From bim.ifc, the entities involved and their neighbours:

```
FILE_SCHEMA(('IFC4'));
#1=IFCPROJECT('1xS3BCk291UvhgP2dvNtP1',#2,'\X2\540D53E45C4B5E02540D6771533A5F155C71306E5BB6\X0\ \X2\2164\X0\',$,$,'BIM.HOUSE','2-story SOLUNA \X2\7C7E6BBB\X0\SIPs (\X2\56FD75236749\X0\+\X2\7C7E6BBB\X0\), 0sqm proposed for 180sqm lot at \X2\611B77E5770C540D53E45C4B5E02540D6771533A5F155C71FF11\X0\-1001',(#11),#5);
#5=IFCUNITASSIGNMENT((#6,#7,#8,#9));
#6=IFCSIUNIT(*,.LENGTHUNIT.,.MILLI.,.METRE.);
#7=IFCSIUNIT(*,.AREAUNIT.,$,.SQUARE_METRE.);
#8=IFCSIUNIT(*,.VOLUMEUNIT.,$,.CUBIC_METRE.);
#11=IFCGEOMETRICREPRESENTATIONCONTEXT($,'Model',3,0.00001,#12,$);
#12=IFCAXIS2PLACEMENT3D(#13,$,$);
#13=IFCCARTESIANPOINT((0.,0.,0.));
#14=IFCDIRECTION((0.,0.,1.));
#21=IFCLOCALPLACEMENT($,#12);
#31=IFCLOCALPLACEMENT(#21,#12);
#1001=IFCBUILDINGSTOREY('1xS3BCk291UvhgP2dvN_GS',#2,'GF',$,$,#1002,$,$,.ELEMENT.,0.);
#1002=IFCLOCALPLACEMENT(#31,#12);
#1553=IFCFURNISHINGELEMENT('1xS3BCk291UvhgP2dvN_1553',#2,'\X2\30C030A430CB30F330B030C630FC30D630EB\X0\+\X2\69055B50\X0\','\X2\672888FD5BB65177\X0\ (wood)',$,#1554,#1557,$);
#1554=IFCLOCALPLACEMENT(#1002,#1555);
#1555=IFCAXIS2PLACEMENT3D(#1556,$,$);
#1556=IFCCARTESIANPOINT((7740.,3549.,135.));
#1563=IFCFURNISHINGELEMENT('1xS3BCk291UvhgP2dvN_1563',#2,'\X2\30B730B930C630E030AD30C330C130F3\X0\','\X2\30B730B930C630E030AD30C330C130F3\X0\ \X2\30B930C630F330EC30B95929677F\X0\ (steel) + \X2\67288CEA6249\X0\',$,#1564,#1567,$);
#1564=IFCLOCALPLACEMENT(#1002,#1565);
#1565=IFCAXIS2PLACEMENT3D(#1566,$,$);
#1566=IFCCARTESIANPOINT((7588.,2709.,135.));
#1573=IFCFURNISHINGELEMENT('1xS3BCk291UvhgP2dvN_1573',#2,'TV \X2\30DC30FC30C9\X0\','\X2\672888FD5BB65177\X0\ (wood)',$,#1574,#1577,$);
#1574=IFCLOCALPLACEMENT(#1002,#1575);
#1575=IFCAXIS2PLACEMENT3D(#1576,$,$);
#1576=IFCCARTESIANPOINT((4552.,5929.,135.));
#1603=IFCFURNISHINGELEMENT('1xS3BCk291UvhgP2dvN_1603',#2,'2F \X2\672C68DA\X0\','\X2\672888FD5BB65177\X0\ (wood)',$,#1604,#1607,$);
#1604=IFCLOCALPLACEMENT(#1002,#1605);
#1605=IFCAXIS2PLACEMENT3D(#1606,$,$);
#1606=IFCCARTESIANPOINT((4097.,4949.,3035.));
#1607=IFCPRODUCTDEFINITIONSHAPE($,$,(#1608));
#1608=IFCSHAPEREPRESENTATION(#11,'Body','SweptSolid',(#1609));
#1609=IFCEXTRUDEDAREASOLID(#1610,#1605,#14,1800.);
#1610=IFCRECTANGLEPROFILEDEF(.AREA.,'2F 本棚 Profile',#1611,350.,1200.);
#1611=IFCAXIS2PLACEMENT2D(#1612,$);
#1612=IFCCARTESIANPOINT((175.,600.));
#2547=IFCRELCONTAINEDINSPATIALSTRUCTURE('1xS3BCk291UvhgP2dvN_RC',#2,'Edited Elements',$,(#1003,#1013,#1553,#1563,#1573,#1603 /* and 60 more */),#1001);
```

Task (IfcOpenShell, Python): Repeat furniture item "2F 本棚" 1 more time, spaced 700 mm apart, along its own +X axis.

```python
import ifcopenshell
import ifcopenshell.api.geometry
import ifcopenshell.api.root
import ifcopenshell.util.element
import ifcopenshell.util.placement
import ifcopenshell.util.unit

model = ifcopenshell.open("bim.ifc")
unit_scale = ifcopenshell.util.unit.calculate_unit_scale(model)


def reuse_history(source, copy):
    """copy_class also copies each property set's owner history, people and application; keep the originals."""
    for rel in copy.IsDefinedBy:
        if rel.is_a("IfcRelDefinesByProperties") and (history := rel.RelatingPropertyDefinition.OwnerHistory):
            rel.RelatingPropertyDefinition.OwnerHistory = source.OwnerHistory
            ifcopenshell.util.element.remove_deep2(model, history)


source = model.by_guid("1xS3BCk291UvhgP2dvN_1603")
base = ifcopenshell.util.placement.get_local_placement(source.ObjectPlacement)
step = base[:3, 0] * 0.7 / unit_scale

for i in range(1, 2):
    copy = ifcopenshell.api.root.copy_class(model, product=source)
    copy.Representation = ifcopenshell.util.element.copy_deep(
        model, source.Representation, exclude=["IfcGeometricRepresentationContext", "IfcRepresentationMap"]
    )
    reuse_history(source, copy)
    matrix = base.copy()
    matrix[:3, 3] += i * step
    print("added at", matrix[:3, 3].round(3) + 0.0)
    ifcopenshell.api.geometry.edit_object_placement(model, product=copy, matrix=matrix, is_si=False)

model.write("bim_edited.ifc")
```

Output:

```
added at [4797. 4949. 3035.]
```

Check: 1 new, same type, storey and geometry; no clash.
